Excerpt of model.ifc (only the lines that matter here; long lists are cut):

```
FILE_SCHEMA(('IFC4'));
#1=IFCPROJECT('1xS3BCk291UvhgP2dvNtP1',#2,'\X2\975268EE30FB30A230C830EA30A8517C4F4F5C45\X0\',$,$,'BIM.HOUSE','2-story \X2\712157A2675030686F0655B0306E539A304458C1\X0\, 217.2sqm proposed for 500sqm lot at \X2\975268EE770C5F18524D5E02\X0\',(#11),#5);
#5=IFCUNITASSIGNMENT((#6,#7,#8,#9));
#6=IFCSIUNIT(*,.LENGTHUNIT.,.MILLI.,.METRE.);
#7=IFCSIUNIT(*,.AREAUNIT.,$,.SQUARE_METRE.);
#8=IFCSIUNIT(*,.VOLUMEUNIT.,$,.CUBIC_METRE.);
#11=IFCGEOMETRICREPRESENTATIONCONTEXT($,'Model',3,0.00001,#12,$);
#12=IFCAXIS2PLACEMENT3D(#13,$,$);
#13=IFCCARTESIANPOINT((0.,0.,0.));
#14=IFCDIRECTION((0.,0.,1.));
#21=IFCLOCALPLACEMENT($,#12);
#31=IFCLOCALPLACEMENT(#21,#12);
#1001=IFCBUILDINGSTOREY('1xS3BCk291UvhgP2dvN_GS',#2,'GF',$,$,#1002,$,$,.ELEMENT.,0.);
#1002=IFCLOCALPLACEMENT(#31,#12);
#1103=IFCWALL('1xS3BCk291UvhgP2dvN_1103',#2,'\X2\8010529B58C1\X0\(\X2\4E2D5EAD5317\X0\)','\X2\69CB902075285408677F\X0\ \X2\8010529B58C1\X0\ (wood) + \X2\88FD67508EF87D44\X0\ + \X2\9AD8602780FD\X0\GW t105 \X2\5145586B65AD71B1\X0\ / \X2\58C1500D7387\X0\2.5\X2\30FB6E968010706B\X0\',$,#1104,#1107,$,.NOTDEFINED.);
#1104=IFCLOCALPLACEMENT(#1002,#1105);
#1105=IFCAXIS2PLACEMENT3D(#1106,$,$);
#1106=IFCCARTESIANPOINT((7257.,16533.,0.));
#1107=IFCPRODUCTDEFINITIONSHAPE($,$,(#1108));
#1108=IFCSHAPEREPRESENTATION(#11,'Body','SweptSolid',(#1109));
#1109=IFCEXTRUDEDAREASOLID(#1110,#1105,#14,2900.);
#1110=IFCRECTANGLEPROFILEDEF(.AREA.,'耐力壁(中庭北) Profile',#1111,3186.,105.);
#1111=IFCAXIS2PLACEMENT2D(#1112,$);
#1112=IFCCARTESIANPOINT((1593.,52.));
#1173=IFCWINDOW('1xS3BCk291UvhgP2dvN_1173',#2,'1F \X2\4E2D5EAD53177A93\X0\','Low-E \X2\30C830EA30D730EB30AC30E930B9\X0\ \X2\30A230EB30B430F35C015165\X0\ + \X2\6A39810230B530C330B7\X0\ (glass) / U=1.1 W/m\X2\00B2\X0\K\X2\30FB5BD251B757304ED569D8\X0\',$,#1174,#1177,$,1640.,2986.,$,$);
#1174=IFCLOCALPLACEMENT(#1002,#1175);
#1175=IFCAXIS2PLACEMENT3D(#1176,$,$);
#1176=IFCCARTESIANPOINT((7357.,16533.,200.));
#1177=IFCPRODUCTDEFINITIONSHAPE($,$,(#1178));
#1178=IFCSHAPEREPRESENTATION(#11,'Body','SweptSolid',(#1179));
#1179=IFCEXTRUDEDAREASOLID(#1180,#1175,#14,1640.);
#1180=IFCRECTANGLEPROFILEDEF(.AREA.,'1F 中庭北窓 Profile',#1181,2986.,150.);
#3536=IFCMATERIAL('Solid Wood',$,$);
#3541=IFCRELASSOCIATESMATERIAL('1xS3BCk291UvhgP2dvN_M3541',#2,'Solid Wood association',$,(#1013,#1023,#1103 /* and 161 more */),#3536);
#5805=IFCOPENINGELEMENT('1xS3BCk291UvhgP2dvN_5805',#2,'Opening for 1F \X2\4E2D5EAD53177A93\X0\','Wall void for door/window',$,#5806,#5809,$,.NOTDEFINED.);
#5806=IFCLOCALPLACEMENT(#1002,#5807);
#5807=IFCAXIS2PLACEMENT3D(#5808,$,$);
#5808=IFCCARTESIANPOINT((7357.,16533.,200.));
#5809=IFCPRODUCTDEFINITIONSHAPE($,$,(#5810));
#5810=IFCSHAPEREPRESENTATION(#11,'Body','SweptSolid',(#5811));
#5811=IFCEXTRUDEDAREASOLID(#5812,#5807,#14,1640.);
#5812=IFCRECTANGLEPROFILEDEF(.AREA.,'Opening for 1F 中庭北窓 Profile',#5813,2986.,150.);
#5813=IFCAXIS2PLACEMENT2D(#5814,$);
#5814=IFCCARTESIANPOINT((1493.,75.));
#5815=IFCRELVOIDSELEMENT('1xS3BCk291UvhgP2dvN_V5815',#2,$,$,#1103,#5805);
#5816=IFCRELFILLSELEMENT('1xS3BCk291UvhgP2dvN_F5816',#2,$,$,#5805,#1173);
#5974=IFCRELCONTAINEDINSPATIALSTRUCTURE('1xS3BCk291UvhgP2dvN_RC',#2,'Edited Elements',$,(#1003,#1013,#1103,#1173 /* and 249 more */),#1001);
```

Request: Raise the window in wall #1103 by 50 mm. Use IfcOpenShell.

```python
import numpy as np
import ifcopenshell
import ifcopenshell.api.geometry
import ifcopenshell.util.placement
import ifcopenshell.util.unit

model = ifcopenshell.open("model.ifc")
unit_scale = ifcopenshell.util.unit.calculate_unit_scale(model)

window = model.by_guid("1xS3BCk291UvhgP2dvN_1173")
opening = window.FillsVoids[0].RelatingOpeningElement
dz = 0.05 / unit_scale

shift = np.array([0.0, 0.0, dz])
# The window is not placed relative to its opening, so move both.
for product in (opening, window):
    matrix = ifcopenshell.util.placement.get_local_placement(product.ObjectPlacement)
    matrix[:3, 3] += shift
    ifcopenshell.api.geometry.edit_object_placement(model, product=product, matrix=matrix, is_si=False)

print(f"moved by {dz * unit_scale:+.3f} m")

model.write("model_v2.ifc")
```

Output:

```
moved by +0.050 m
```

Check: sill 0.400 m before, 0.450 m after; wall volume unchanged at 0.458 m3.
